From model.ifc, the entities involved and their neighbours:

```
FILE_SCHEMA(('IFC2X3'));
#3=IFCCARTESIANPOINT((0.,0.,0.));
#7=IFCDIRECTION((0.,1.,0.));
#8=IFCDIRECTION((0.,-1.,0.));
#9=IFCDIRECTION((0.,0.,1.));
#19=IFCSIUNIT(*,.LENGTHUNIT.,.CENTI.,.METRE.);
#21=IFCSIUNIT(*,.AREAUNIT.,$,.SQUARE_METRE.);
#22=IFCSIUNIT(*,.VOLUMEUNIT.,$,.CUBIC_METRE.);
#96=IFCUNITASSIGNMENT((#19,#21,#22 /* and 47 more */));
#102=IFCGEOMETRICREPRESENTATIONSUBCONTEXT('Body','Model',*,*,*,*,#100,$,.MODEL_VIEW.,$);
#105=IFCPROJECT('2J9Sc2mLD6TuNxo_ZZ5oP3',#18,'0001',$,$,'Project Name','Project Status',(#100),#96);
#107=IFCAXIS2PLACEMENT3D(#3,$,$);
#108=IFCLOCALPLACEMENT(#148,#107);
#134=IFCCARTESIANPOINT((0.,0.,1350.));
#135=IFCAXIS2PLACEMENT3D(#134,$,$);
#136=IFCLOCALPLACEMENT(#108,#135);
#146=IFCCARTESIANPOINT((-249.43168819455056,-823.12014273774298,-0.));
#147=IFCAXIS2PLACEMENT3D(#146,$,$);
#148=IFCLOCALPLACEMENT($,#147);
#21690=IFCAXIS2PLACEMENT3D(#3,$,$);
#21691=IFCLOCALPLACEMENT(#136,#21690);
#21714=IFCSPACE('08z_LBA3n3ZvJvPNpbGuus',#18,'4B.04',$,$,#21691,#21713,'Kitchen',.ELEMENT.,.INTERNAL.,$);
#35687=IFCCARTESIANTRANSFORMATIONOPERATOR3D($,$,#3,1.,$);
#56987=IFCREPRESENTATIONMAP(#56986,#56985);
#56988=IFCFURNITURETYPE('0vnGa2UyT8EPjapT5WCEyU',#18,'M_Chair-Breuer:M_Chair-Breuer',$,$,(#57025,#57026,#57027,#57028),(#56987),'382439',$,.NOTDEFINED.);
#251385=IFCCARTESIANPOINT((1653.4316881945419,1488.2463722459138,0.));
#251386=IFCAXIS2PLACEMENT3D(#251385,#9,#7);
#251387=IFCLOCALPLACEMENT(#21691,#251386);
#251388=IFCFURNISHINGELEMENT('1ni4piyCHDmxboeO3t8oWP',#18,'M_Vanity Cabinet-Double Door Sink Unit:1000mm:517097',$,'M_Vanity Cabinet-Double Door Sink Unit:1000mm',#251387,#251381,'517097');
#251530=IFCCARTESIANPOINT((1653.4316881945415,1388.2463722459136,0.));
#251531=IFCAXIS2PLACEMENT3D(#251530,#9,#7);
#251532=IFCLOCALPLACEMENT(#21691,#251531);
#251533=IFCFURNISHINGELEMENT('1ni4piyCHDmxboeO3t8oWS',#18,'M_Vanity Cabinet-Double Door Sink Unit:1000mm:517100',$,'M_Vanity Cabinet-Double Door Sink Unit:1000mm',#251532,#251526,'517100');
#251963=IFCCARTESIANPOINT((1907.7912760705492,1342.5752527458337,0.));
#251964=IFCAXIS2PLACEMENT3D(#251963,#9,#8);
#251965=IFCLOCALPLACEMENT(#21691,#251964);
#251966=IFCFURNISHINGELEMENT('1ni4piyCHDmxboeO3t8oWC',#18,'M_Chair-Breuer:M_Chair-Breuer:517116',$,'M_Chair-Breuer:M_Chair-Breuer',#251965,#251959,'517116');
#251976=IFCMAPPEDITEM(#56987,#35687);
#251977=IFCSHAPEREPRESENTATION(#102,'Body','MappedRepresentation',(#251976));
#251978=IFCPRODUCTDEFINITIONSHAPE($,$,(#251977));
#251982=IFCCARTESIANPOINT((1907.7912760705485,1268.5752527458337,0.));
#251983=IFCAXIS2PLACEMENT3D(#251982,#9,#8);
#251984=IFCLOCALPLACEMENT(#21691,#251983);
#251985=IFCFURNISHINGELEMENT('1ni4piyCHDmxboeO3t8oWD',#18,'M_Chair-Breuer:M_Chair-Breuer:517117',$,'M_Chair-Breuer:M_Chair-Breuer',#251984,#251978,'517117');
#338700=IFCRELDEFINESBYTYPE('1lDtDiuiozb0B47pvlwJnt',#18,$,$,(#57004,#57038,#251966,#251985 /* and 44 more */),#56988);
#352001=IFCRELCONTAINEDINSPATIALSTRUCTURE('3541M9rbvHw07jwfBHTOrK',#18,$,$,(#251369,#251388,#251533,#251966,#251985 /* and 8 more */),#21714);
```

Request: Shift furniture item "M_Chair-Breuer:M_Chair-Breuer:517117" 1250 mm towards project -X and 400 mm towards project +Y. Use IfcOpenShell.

```python
import ifcopenshell
import ifcopenshell.api.geometry
import ifcopenshell.util.placement
import ifcopenshell.util.unit

model = ifcopenshell.open("model.ifc")
unit_scale = ifcopenshell.util.unit.calculate_unit_scale(model)

item = model.by_guid("1ni4piyCHDmxboeO3t8oWD")
matrix = ifcopenshell.util.placement.get_local_placement(item.ObjectPlacement)
matrix[0, 3] -= 1.25 / unit_scale
matrix[1, 3] += 0.4 / unit_scale
ifcopenshell.api.geometry.edit_object_placement(model, product=item, matrix=matrix, is_si=False)

print(ifcopenshell.util.placement.get_local_placement(item.ObjectPlacement).round(3) + 0.0)

model.write("model_rev.ifc")
```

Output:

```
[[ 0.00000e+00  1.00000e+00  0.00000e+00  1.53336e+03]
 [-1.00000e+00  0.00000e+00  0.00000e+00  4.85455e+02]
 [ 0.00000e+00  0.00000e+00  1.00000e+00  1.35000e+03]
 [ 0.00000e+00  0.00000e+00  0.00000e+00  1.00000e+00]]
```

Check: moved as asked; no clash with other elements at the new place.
